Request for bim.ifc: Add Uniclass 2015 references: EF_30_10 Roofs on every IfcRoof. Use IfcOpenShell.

First a look at what the model holds.

```python
import ifcopenshell

model = ifcopenshell.open("bim.ifc")
print(model.schema)
print("classifications:", [c.Name for c in model.by_type("IfcClassification")])
for ifc_class in ("IfcDoor", "IfcRoof", "IfcStair", "IfcWall", "IfcWindow"):
    print(ifc_class, len(model.by_type(ifc_class)))
```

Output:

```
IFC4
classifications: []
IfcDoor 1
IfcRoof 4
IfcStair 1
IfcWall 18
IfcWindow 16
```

```python
import ifcopenshell
import ifcopenshell.api.classification

model = ifcopenshell.open("bim.ifc")

system = ifcopenshell.api.classification.add_classification(model, classification="Uniclass 2015")

codes = {
    "IfcRoof": ("EF_30_10", "Roofs"),
}
for ifc_class, (code, name) in codes.items():
    products = model.by_type(ifc_class)
    ifcopenshell.api.classification.add_reference(
        model, products=products, classification=system, identification=code, name=name
    )
    print(code, len(products))

model.write("bim_updated.ifc")
```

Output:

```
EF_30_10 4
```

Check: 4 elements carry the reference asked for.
